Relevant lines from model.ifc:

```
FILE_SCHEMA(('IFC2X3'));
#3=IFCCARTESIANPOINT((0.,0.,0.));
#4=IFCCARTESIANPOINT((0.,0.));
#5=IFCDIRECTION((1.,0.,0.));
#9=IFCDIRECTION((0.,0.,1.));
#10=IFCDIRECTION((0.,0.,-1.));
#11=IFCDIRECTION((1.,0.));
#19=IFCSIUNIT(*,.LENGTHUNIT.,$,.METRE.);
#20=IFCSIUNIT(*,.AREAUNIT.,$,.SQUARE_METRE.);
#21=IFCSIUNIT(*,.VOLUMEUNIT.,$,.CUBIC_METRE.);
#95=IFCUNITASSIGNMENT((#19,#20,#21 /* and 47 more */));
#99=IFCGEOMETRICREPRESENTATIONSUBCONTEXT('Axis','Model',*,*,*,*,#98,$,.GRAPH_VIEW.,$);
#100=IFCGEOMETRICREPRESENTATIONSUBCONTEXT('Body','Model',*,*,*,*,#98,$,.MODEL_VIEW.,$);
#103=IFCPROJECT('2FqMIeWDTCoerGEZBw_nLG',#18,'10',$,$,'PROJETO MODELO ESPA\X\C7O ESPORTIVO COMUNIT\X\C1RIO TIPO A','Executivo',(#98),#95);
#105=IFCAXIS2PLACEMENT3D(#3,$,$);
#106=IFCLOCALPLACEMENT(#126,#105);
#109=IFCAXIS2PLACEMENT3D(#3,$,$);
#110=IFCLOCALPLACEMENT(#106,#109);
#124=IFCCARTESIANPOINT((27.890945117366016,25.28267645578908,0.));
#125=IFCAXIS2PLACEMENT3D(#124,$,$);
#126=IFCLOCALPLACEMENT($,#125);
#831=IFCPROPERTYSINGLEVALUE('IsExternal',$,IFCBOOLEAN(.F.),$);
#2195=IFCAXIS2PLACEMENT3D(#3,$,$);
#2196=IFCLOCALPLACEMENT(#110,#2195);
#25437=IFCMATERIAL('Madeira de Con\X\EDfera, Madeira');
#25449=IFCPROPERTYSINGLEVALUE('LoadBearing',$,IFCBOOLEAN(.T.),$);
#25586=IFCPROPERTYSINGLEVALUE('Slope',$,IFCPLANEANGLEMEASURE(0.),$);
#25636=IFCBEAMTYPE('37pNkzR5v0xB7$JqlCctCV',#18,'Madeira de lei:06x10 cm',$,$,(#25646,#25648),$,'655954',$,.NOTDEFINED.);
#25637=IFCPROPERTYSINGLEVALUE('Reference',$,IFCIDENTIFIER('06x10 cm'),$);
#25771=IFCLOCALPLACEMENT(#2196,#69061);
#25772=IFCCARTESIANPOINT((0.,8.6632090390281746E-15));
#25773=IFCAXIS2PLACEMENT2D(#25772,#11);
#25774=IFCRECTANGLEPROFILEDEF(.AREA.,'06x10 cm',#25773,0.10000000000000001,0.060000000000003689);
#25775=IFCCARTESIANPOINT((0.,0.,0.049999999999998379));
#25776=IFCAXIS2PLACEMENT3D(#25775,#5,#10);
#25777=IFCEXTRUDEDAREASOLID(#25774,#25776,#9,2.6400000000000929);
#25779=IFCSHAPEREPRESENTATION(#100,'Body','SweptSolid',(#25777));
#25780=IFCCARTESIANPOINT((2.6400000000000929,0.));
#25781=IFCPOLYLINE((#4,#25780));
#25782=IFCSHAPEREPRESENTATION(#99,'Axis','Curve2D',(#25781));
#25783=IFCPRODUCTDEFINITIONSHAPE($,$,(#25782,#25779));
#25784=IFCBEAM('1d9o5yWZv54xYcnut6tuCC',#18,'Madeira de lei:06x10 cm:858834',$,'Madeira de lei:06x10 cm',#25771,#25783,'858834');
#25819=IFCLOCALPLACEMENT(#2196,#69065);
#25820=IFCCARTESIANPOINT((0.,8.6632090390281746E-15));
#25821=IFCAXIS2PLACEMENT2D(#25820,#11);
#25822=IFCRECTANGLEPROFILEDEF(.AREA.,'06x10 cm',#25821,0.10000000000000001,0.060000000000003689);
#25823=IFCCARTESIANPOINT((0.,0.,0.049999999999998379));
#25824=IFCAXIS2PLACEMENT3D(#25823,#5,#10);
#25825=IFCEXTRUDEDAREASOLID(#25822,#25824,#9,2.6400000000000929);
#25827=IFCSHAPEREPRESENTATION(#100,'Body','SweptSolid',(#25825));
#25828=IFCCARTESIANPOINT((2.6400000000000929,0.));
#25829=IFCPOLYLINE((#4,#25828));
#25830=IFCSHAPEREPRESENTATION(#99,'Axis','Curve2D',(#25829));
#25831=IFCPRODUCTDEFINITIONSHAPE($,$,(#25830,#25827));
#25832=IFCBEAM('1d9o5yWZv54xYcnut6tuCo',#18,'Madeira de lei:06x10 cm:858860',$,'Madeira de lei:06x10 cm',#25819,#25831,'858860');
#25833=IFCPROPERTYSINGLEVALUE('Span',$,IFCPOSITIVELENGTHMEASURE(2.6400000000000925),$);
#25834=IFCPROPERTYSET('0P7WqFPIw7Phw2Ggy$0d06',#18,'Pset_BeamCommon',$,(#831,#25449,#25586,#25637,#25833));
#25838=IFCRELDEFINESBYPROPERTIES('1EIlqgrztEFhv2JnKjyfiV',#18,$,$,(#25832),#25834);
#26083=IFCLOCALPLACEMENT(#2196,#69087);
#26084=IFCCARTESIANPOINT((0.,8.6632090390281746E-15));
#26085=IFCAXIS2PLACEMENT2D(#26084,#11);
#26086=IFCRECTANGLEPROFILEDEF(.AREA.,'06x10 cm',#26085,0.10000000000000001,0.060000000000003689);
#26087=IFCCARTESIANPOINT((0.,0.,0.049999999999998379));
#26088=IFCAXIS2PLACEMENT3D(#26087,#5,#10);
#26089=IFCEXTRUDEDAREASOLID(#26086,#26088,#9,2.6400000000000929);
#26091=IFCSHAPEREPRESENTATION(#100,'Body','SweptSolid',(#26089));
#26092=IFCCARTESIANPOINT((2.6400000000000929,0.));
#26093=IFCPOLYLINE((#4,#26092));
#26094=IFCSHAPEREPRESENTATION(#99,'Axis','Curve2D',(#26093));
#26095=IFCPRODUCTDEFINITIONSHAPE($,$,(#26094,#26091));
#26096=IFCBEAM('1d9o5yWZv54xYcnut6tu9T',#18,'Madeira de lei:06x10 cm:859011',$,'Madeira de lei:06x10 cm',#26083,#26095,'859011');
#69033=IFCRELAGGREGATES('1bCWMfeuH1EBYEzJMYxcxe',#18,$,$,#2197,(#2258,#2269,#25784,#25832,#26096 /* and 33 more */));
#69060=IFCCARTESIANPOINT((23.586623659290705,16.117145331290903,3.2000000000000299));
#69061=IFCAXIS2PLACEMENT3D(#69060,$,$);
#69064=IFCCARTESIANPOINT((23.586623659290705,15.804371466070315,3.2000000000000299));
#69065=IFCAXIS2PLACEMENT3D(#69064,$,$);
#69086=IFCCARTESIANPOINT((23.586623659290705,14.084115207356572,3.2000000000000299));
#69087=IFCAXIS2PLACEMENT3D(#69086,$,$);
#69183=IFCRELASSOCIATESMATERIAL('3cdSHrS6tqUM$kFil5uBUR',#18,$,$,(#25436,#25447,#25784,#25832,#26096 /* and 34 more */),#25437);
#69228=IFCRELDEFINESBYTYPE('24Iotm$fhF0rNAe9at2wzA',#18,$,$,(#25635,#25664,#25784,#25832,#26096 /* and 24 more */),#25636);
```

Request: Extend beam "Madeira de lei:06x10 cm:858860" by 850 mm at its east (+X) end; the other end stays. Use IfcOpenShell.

```python
import numpy as np
import ifcopenshell
import ifcopenshell.api.pset
import ifcopenshell.util.element
import ifcopenshell.util.representation
import ifcopenshell.util.unit

model = ifcopenshell.open("model.ifc")
unit_scale = ifcopenshell.util.unit.calculate_unit_scale(model)

member = model.by_guid("1d9o5yWZv54xYcnut6tuCo")
change = 0.85 / unit_scale

# The extrusion runs towards the end named, so only its depth changes.
body = ifcopenshell.util.representation.get_representation(member, "Model", "Body")
solid = body.Items[0]
old_length = solid.Depth
solid.Depth += change

# Move the axis end point with it.
axis = next(r for r in member.Representation.Representations if r.RepresentationIdentifier == "Axis").Items[0]
start, end = (np.array(p.Coordinates) for p in axis.Points)
end = end + (end - start) / np.linalg.norm(end - start) * change
point = model.createIfcCartesianPoint(end.tolist())
axis.Points = [axis.Points[0], point]

# Update the stored length and volume.
pset = model.by_id(ifcopenshell.util.element.get_pset(member, "Pset_BeamCommon", should_inherit=False)["id"])
ifcopenshell.api.pset.edit_pset(model, pset=pset, properties={
    "Span": model.create_entity("IfcPositiveLengthMeasure", solid.Depth),
})

print(f"length {old_length:g} -> {solid.Depth:g}")

model.write("model_rev.ifc")
```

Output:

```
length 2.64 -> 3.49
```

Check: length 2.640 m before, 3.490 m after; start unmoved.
